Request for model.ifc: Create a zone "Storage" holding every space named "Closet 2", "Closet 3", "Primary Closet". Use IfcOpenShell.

First a look at what the model holds.

```python
import ifcopenshell

model = ifcopenshell.open("model.ifc")
print(model.schema)
seen = {}
for space in model.by_type("IfcSpace"):
    seen[space.LongName] = seen.get(space.LongName, 0) + 1
for name, count in sorted(seen.items(), key=str):
    print(count, "x", name)
print("zones:", [z.Name for z in model.by_type("IfcZone")][:20])
```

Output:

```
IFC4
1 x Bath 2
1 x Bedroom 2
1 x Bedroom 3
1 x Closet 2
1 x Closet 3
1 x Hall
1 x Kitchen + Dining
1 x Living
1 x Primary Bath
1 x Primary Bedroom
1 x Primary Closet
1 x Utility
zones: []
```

```python
import ifcopenshell
import ifcopenshell.api.group
import ifcopenshell.api.root

model = ifcopenshell.open("model.ifc")

names = {"Closet 2", "Closet 3", "Primary Closet"}
spaces = [s for s in model.by_type("IfcSpace") if s.LongName in names]

zone = ifcopenshell.api.root.create_entity(model, ifc_class="IfcZone", name="Storage")
ifcopenshell.api.group.assign_group(model, products=spaces, group=zone)
print(len(spaces), "spaces in", zone.Name)

model.write("model-out.ifc")
```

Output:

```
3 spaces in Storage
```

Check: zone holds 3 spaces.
